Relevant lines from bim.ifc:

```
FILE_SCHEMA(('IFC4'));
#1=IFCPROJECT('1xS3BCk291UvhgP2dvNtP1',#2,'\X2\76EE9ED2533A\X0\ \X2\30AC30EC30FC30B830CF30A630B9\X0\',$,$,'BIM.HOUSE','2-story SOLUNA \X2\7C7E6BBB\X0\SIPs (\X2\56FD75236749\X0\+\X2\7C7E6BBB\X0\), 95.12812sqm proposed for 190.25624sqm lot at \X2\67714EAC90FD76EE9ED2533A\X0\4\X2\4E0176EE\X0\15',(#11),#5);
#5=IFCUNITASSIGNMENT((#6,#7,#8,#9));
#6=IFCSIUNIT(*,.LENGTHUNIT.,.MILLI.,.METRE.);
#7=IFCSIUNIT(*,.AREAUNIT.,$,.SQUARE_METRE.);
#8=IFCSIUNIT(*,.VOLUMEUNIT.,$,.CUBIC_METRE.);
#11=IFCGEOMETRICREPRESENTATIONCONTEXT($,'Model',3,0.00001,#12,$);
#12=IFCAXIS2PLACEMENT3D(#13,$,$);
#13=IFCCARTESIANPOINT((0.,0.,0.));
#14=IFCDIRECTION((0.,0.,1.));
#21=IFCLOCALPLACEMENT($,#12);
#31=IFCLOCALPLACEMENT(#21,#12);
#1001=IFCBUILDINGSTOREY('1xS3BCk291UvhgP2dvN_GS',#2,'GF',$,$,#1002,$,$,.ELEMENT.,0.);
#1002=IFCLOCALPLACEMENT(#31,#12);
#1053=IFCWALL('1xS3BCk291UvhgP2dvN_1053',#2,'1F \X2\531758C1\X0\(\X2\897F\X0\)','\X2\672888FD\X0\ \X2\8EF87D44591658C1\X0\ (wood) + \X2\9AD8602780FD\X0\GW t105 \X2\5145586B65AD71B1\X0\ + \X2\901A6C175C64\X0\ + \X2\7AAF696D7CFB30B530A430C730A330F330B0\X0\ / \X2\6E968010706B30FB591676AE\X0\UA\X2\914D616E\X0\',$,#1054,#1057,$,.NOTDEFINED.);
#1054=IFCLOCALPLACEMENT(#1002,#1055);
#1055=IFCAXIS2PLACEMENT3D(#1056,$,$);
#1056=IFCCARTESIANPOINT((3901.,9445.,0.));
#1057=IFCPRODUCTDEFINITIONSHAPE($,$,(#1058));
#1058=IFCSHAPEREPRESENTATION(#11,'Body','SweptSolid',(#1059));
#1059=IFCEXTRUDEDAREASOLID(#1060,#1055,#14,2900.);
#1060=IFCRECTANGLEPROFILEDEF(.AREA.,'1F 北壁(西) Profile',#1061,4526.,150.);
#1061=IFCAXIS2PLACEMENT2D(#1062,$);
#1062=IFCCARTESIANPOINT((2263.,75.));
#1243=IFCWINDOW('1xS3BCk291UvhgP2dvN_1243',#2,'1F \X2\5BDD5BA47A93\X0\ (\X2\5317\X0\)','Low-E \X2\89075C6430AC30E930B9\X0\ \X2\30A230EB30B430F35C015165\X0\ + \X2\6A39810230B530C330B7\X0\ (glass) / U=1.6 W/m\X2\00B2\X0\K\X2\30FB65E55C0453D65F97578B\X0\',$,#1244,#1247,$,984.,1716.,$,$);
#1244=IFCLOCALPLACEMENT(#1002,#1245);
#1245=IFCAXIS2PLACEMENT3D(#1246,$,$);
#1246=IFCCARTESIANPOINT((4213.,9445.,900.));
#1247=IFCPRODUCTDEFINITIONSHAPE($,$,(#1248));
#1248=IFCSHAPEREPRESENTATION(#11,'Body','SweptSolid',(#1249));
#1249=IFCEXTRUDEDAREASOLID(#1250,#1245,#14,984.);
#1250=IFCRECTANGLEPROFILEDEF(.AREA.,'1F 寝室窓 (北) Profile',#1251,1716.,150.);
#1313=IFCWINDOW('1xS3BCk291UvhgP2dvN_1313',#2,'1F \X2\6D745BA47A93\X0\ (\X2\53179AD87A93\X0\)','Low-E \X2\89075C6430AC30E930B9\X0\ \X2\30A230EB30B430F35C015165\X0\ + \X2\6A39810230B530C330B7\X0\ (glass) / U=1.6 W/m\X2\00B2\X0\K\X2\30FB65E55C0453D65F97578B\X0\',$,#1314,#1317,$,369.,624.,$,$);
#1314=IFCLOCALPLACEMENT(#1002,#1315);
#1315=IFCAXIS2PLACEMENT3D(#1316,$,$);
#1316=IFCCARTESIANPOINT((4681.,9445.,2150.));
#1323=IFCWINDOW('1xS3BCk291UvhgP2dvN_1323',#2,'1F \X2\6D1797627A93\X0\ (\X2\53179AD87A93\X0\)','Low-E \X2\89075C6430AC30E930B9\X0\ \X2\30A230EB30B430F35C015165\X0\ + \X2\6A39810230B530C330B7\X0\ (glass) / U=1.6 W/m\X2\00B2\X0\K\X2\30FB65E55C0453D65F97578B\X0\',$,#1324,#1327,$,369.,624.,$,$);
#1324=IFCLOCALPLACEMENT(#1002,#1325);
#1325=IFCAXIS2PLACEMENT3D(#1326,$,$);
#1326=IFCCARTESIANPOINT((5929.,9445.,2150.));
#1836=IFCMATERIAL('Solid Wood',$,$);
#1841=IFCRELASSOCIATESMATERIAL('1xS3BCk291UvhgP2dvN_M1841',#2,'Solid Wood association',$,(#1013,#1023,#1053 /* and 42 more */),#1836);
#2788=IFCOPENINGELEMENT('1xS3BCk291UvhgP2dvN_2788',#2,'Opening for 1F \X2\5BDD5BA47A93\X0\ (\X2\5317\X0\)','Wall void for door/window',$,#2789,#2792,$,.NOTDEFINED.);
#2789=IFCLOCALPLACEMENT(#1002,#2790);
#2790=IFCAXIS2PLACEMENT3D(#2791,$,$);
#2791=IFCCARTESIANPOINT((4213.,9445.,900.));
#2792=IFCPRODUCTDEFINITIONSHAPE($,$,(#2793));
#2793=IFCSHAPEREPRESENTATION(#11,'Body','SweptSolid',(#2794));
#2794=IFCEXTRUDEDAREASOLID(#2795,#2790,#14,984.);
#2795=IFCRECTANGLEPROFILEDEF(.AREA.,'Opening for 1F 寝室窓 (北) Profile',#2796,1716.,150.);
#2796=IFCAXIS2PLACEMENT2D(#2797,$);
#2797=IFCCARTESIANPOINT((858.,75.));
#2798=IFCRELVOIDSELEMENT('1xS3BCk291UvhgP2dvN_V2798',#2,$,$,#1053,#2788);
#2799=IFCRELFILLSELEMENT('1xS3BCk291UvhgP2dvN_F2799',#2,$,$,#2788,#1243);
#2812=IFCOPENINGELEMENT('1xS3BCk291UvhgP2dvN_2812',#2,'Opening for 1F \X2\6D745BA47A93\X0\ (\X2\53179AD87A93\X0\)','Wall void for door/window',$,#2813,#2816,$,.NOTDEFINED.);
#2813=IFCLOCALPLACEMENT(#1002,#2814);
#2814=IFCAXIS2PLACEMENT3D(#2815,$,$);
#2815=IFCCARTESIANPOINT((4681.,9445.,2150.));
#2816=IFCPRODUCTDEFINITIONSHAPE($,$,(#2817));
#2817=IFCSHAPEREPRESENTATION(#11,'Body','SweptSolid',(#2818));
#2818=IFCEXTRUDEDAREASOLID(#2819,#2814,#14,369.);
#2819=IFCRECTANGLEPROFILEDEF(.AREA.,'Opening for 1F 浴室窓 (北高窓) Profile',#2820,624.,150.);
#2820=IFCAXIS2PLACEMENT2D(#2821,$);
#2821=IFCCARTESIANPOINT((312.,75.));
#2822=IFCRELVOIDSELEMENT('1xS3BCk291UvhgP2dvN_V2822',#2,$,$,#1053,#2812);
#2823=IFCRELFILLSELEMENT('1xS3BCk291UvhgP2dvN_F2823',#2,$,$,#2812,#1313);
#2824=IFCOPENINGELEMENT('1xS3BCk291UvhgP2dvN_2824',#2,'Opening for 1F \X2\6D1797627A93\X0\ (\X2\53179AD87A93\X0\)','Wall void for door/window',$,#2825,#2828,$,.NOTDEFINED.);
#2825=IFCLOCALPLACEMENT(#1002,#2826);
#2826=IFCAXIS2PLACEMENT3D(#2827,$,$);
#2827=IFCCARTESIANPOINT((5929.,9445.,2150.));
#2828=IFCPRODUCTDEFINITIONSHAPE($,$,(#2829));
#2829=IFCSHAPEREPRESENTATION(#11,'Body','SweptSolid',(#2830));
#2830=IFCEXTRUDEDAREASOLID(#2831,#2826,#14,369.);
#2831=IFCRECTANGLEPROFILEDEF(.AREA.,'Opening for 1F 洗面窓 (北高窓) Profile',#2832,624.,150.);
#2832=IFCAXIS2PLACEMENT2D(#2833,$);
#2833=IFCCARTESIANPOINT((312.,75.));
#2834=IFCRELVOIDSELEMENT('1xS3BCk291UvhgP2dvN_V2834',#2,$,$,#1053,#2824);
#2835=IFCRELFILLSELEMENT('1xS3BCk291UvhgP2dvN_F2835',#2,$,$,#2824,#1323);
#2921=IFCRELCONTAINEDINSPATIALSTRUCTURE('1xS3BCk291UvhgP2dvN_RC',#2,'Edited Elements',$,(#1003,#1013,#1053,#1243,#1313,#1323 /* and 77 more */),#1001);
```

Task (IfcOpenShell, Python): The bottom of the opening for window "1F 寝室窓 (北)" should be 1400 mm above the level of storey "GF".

```python
import numpy as np
import ifcopenshell
import ifcopenshell.api.geometry
import ifcopenshell.geom
import ifcopenshell.util.element
import ifcopenshell.util.placement
import ifcopenshell.util.shape
import ifcopenshell.util.unit

model = ifcopenshell.open("bim.ifc")
unit_scale = ifcopenshell.util.unit.calculate_unit_scale(model)

window = model.by_id(1243)
opening = window.FillsVoids[0].RelatingOpeningElement
storey = ifcopenshell.util.element.get_container(window, ifc_class="IfcBuildingStorey")
level = ifcopenshell.util.placement.get_local_placement(storey.ObjectPlacement)[2, 3]

# The opening's origin need not be at the sill, so measure its lowest point.
shape = ifcopenshell.geom.create_shape(ifcopenshell.geom.settings(), opening)
bottom = ifcopenshell.util.shape.get_shape_bottom_elevation(shape, shape.geometry) / unit_scale
dz = level + 1400.0 - bottom

shift = np.array([0.0, 0.0, dz])
# The window is not placed relative to its opening, so move both.
for product in (opening, window):
    matrix = ifcopenshell.util.placement.get_local_placement(product.ObjectPlacement)
    matrix[:3, 3] += shift
    ifcopenshell.api.geometry.edit_object_placement(model, product=product, matrix=matrix, is_si=False)

print(f"moved by {dz * unit_scale:+.3f} m")

model.write("bim-out.ifc")
```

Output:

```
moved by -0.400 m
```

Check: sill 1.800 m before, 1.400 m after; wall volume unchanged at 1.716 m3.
